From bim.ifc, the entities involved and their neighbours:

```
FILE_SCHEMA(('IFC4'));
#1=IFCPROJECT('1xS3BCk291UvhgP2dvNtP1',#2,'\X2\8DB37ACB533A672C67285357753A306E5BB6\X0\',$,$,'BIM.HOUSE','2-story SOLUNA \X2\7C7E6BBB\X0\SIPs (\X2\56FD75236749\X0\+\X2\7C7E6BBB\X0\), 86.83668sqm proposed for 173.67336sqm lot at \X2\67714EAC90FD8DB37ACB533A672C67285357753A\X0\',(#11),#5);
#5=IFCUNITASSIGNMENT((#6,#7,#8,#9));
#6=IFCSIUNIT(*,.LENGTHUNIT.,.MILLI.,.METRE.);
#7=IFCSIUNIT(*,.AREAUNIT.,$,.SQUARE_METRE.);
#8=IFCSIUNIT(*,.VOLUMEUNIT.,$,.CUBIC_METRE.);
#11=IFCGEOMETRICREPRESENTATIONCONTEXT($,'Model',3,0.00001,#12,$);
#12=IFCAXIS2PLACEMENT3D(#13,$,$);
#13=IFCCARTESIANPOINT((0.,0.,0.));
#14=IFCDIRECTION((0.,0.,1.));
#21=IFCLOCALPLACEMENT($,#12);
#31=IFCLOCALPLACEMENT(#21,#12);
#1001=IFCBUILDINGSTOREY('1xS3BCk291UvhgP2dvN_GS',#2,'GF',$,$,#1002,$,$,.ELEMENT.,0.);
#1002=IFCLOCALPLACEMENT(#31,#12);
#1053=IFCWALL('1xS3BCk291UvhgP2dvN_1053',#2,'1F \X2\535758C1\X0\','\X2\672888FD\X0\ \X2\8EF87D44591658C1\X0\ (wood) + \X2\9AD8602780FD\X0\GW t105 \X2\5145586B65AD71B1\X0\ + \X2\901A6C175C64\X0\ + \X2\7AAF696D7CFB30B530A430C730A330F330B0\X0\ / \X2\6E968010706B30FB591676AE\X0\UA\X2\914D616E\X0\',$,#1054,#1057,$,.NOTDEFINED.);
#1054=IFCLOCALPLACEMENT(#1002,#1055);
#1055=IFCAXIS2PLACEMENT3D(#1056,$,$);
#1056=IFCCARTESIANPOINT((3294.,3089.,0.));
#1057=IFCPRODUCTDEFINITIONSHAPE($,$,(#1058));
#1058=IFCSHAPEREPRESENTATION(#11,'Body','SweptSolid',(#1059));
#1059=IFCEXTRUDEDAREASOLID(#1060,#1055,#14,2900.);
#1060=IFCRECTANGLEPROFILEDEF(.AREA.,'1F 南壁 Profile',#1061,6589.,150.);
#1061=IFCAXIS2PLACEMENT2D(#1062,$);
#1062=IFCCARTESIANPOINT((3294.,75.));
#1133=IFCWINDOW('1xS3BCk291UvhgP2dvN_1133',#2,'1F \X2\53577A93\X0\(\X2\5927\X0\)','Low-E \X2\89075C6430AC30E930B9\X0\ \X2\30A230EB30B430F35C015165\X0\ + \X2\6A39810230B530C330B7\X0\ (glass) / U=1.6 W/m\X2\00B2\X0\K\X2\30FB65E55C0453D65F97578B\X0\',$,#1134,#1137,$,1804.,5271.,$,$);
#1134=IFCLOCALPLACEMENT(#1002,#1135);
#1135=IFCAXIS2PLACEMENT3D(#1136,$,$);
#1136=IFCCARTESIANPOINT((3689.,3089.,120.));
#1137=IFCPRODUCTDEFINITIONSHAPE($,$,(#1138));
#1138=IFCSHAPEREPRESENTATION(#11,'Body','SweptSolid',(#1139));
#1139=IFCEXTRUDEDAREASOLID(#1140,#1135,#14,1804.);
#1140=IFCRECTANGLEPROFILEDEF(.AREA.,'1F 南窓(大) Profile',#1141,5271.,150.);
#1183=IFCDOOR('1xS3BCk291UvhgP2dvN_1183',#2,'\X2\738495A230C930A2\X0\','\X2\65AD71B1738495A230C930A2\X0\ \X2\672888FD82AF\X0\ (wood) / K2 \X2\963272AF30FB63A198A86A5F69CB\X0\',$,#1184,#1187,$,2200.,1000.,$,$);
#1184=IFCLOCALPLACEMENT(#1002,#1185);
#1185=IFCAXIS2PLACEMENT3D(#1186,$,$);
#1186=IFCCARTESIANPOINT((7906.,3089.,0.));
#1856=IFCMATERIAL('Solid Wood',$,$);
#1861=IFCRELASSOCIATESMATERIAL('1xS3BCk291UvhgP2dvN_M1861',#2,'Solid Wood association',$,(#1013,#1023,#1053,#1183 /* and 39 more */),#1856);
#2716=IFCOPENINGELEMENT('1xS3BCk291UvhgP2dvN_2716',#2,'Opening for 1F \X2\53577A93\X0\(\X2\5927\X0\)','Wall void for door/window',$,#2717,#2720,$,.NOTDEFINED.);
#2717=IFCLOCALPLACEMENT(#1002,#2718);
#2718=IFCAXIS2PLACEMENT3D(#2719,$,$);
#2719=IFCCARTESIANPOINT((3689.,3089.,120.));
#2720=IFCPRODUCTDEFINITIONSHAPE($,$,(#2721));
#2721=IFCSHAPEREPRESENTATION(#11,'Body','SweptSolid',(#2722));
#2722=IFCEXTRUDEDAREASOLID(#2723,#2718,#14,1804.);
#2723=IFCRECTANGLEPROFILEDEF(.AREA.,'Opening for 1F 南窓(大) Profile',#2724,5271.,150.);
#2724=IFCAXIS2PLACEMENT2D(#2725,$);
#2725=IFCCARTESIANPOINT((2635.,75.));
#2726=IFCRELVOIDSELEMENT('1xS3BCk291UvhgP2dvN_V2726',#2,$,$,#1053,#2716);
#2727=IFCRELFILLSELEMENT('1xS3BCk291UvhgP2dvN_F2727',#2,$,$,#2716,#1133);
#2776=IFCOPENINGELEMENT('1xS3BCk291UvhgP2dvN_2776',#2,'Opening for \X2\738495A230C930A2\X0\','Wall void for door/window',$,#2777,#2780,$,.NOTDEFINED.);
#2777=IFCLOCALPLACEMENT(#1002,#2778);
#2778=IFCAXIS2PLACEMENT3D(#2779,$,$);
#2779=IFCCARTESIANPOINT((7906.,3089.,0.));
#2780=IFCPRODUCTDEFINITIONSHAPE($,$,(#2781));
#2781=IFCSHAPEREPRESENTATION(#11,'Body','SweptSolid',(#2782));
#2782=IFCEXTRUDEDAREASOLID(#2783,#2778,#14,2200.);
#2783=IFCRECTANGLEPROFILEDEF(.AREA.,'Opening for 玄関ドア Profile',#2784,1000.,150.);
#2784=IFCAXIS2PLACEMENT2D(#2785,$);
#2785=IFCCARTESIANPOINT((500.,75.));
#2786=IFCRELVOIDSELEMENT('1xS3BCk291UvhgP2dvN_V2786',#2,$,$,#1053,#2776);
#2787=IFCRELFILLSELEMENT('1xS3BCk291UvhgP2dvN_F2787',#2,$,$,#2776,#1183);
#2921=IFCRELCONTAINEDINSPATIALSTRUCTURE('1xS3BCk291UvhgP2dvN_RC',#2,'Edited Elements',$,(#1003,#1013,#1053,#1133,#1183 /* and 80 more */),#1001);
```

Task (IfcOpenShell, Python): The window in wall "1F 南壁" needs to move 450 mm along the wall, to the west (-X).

```python
import ifcopenshell
import ifcopenshell.api.geometry
import ifcopenshell.util.placement

model = ifcopenshell.open("bim.ifc")

window = model.by_guid("1xS3BCk291UvhgP2dvN_1133")
opening = window.FillsVoids[0].RelatingOpeningElement
wall = opening.VoidsElements[0].RelatingBuildingElement

wall_matrix = ifcopenshell.util.placement.get_local_placement(wall.ObjectPlacement)
shift = wall_matrix[:3, 0] * -450.0
before = ifcopenshell.util.placement.get_local_placement(window.ObjectPlacement)[:3, 3].copy()

# The window is not placed relative to its opening, so move both.
for product in (opening, window):
    matrix = ifcopenshell.util.placement.get_local_placement(product.ObjectPlacement)
    matrix[:3, 3] += shift
    ifcopenshell.api.geometry.edit_object_placement(model, product=product, matrix=matrix, is_si=False)

after = ifcopenshell.util.placement.get_local_placement(window.ObjectPlacement)[:3, 3]
print("window moved by", (after - before).round(3) + 0.0)

model.write("bim-out.ifc")
```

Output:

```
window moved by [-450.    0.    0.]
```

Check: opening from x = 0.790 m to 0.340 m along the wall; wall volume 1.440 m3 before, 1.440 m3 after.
